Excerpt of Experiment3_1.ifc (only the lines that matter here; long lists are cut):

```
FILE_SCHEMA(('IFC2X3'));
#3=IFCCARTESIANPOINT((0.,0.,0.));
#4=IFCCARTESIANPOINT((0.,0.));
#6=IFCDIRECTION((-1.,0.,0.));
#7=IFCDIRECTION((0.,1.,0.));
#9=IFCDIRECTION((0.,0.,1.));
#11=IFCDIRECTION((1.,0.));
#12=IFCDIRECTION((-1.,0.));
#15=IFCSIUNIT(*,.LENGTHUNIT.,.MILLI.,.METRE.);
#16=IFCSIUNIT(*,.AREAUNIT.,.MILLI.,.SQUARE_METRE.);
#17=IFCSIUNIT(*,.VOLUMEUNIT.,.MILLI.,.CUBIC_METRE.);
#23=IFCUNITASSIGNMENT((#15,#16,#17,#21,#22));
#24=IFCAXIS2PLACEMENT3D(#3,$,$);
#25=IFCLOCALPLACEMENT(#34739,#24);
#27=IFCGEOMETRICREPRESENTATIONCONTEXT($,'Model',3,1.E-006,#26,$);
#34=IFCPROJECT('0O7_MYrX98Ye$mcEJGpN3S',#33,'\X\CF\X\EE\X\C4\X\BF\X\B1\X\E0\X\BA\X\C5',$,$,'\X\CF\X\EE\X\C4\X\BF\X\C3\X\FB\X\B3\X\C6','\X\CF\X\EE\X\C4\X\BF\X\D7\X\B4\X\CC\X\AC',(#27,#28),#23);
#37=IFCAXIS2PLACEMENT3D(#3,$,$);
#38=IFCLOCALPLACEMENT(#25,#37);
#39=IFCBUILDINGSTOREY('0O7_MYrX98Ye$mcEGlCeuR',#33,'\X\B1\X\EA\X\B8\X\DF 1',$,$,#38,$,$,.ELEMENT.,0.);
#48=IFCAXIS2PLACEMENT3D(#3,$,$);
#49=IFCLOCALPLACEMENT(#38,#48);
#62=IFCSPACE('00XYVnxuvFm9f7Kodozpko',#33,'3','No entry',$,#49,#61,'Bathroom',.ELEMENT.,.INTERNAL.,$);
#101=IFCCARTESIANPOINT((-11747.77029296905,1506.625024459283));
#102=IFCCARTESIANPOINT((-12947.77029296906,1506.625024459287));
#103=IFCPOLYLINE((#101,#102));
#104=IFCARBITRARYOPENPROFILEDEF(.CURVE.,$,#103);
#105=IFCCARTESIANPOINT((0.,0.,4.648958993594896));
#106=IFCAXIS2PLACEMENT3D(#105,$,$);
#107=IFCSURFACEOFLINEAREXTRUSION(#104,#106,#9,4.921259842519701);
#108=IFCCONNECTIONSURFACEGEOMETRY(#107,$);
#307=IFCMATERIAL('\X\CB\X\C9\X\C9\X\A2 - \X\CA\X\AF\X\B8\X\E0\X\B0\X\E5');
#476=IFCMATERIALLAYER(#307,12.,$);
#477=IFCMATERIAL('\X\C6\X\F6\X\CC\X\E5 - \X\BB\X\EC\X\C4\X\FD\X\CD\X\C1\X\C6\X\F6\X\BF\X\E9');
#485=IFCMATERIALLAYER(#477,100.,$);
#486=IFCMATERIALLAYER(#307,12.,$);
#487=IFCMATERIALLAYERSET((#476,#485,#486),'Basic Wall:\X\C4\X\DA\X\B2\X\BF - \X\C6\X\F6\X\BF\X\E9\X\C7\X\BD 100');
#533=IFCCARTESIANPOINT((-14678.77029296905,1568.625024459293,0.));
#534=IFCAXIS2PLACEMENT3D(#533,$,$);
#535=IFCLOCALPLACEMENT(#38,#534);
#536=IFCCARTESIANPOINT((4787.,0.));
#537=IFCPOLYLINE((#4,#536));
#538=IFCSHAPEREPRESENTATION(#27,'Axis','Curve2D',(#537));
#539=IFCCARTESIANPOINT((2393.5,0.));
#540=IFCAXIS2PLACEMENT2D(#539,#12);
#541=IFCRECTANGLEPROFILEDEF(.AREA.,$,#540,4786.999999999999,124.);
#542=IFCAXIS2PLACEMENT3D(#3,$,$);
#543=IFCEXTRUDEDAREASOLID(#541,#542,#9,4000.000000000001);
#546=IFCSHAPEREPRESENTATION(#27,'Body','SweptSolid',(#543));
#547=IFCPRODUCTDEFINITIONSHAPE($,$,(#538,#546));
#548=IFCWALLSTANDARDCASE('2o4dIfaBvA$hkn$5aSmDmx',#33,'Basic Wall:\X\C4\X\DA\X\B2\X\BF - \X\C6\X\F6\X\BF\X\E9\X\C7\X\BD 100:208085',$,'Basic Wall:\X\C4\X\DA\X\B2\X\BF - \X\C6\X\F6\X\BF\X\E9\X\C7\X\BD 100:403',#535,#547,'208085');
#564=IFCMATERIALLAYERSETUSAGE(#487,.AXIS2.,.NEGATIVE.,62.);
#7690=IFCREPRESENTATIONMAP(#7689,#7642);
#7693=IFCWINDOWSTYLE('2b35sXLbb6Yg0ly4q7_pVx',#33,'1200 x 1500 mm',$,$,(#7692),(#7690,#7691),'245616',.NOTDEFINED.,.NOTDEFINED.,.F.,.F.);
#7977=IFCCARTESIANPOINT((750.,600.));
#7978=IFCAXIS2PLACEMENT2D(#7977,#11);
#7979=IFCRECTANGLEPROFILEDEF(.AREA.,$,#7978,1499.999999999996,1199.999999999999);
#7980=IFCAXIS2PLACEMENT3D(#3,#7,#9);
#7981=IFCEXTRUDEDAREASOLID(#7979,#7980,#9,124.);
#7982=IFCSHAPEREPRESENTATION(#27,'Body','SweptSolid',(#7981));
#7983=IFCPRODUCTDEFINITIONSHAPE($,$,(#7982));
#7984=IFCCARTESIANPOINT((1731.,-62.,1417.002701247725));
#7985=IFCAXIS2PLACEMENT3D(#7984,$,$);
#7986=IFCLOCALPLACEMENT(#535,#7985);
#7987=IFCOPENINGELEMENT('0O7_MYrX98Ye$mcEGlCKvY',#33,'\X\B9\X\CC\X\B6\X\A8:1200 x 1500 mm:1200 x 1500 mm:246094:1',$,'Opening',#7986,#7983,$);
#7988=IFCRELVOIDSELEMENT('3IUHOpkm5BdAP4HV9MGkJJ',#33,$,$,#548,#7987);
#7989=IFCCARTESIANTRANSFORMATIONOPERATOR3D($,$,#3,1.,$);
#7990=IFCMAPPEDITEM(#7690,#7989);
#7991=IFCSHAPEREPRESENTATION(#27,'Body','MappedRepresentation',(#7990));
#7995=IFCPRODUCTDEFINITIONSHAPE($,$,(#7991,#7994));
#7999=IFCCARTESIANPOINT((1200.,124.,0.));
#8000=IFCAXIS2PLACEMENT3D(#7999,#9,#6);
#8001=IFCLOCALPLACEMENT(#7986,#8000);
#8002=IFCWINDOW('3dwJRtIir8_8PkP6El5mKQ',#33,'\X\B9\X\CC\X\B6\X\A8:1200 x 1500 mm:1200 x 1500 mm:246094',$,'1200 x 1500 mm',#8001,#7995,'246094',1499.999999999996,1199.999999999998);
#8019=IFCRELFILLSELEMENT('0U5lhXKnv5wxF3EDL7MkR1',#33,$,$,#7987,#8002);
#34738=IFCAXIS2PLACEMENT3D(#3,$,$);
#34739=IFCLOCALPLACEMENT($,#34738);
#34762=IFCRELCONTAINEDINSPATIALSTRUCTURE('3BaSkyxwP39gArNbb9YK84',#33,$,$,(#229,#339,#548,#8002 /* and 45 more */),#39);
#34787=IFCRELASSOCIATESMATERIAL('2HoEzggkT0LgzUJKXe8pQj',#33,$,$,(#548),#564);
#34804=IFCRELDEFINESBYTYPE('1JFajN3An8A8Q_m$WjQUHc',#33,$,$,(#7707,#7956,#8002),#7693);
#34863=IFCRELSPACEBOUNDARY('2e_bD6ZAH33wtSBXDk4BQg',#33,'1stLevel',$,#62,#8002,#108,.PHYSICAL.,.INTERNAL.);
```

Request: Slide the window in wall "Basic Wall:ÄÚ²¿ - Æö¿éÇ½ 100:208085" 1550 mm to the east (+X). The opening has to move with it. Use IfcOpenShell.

```python
import numpy as np
import ifcopenshell
import ifcopenshell.api.geometry
import ifcopenshell.util.placement

model = ifcopenshell.open("Experiment3_1.ifc")

window = model.by_guid("3dwJRtIir8_8PkP6El5mKQ")
opening = window.FillsVoids[0].RelatingOpeningElement
wall = opening.VoidsElements[0].RelatingBuildingElement

wall_matrix = ifcopenshell.util.placement.get_local_placement(wall.ObjectPlacement)
shift = wall_matrix[:3, 0] * 1550.0
before = ifcopenshell.util.placement.get_local_placement(window.ObjectPlacement)[:3, 3].copy()

# The window is placed relative to its opening, so it follows when the opening moves.
matrix = ifcopenshell.util.placement.get_local_placement(opening.ObjectPlacement)
matrix[:3, 3] += shift
ifcopenshell.api.geometry.edit_object_placement(
    model, product=opening, matrix=matrix, is_si=False, should_transform_children=True
)

# Space boundary surfaces are stored in each space's coordinates; move them too.
for rel in window.ProvidesBoundaries:
    if not rel.ConnectionGeometry:
        continue
    surface = rel.ConnectionGeometry.SurfaceOnRelatingElement
    space_matrix = ifcopenshell.util.placement.get_local_placement(rel.RelatingSpace.ObjectPlacement)
    point = np.array(surface.Position.Location.Coordinates) + space_matrix[:3, :3].T @ shift
    surface.Position = model.createIfcAxis2Placement3D(
        model.createIfcCartesianPoint(point.tolist()), surface.Position.Axis, surface.Position.RefDirection
    )

after = ifcopenshell.util.placement.get_local_placement(window.ObjectPlacement)[:3, 3]
print("window moved by", (after - before).round(3) + 0.0)

model.write("Experiment3_1_v2.ifc")
```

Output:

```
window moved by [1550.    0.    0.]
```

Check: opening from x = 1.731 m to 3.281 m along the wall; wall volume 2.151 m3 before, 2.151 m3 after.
